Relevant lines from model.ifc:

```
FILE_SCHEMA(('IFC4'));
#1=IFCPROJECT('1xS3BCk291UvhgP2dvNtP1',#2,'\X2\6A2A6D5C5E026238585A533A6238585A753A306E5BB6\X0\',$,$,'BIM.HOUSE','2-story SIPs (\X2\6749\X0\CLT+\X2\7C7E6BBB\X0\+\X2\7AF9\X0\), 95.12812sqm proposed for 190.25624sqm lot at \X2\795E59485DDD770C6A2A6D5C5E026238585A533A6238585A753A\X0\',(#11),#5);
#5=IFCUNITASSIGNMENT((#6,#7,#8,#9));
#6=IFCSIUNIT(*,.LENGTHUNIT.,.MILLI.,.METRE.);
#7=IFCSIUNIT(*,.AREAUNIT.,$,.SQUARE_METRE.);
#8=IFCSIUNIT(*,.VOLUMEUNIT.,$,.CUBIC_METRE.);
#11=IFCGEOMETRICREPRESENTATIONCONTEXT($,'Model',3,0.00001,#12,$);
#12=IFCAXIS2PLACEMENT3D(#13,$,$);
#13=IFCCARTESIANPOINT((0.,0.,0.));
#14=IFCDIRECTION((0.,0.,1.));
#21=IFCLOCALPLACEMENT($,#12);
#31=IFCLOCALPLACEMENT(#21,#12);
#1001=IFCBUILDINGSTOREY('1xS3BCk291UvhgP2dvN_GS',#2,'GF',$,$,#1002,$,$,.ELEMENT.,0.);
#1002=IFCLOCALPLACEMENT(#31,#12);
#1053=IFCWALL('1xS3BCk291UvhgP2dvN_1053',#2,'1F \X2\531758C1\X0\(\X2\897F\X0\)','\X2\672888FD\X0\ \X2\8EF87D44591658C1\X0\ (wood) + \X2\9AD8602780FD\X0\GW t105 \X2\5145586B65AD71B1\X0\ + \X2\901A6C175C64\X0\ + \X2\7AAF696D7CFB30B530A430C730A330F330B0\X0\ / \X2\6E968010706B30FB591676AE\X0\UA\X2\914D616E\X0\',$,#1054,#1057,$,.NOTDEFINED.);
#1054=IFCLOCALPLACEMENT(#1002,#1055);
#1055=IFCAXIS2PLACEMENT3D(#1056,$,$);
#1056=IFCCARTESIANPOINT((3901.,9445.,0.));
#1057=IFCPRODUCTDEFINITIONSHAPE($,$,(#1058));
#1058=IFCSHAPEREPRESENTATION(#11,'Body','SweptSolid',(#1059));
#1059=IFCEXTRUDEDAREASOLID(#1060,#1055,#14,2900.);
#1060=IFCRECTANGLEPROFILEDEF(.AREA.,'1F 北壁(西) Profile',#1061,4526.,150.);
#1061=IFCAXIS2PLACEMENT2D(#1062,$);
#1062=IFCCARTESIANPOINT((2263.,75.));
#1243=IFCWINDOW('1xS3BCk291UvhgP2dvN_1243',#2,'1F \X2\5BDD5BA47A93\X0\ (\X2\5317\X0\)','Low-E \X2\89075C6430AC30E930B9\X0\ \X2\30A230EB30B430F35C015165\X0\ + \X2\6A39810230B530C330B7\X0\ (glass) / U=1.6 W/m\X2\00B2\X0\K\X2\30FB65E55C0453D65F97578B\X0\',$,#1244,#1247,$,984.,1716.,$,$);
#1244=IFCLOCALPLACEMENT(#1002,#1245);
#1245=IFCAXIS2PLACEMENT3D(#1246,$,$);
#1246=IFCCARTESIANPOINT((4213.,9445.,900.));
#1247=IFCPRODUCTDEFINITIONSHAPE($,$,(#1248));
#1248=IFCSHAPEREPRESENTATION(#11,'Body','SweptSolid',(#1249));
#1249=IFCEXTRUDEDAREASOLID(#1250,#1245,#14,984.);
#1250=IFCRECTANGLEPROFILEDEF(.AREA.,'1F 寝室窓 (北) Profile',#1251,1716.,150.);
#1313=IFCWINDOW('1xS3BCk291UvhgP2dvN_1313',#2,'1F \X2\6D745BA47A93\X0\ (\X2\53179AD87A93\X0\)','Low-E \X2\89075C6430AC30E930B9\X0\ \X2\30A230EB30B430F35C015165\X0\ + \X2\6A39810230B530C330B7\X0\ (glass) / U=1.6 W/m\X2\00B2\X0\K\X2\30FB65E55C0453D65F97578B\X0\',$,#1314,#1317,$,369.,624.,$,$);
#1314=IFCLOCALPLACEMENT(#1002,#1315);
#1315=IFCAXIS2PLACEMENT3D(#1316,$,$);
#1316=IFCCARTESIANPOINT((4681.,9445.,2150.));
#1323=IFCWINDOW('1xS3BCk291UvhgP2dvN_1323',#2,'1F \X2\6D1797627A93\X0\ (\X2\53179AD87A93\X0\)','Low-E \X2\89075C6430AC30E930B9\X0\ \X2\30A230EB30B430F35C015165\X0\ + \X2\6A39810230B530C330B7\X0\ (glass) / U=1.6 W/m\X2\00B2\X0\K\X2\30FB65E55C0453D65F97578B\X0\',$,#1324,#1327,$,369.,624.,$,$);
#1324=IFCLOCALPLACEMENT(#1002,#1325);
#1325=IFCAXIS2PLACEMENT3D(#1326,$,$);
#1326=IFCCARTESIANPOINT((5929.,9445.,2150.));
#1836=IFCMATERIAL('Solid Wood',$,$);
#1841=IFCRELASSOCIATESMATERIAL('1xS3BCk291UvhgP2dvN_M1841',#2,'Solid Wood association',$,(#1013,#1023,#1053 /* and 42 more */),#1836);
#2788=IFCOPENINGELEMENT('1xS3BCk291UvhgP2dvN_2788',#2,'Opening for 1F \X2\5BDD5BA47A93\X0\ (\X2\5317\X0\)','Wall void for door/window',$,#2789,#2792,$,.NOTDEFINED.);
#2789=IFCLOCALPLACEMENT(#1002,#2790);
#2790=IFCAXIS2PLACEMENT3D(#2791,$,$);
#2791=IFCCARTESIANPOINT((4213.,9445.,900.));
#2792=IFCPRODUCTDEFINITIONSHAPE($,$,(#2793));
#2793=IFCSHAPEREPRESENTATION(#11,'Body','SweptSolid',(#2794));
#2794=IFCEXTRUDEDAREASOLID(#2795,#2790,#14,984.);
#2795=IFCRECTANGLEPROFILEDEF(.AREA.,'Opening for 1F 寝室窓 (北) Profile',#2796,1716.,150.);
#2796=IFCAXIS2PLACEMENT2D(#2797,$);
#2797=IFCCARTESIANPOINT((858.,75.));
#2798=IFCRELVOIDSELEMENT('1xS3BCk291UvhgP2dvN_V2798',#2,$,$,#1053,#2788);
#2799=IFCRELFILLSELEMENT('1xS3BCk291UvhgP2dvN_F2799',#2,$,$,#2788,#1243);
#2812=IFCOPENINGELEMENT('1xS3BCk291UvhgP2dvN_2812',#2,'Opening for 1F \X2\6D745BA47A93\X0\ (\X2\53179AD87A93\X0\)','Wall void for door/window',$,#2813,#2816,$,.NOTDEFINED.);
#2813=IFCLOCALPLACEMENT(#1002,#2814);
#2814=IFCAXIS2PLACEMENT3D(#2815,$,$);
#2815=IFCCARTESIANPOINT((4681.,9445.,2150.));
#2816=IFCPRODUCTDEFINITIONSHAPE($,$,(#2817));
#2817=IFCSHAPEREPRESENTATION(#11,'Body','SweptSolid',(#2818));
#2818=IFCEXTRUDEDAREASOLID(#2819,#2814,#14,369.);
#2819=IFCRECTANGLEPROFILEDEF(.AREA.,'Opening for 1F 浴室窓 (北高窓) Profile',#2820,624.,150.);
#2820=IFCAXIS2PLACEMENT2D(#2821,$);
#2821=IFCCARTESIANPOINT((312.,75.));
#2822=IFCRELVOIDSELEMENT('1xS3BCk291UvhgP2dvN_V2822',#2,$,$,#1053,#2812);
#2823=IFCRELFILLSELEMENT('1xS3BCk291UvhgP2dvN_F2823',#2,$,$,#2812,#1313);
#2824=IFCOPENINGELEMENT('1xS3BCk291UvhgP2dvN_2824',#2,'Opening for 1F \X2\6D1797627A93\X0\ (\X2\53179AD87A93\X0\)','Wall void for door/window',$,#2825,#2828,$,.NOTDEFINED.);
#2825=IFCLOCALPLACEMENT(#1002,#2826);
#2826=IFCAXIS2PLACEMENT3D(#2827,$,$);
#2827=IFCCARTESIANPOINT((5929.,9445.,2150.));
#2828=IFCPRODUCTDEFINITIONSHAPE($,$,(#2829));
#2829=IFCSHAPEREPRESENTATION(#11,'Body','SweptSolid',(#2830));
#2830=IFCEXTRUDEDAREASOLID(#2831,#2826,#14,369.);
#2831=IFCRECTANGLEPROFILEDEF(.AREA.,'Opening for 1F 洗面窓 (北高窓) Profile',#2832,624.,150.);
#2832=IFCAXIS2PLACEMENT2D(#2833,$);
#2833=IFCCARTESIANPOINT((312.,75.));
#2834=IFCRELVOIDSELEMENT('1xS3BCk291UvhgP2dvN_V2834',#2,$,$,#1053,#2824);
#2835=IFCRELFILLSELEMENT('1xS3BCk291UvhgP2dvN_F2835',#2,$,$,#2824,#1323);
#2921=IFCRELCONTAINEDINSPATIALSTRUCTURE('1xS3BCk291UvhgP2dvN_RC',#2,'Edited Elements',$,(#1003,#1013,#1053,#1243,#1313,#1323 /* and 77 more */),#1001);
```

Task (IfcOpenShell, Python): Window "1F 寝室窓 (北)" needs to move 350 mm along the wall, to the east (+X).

```python
import ifcopenshell
import ifcopenshell.api.geometry
import ifcopenshell.util.placement
import ifcopenshell.util.unit

model = ifcopenshell.open("model.ifc")
unit_scale = ifcopenshell.util.unit.calculate_unit_scale(model)

window = model.by_guid("1xS3BCk291UvhgP2dvN_1243")
opening = window.FillsVoids[0].RelatingOpeningElement
wall = opening.VoidsElements[0].RelatingBuildingElement

wall_matrix = ifcopenshell.util.placement.get_local_placement(wall.ObjectPlacement)
shift = wall_matrix[:3, 0] * 0.35 / unit_scale
before = ifcopenshell.util.placement.get_local_placement(window.ObjectPlacement)[:3, 3].copy()

# The window is not placed relative to its opening, so move both.
for product in (opening, window):
    matrix = ifcopenshell.util.placement.get_local_placement(product.ObjectPlacement)
    matrix[:3, 3] += shift
    ifcopenshell.api.geometry.edit_object_placement(model, product=product, matrix=matrix, is_si=False)

after = ifcopenshell.util.placement.get_local_placement(window.ObjectPlacement)[:3, 3]
print("window moved by", (after - before).round(3) + 0.0)

model.write("model_v2.ifc")
```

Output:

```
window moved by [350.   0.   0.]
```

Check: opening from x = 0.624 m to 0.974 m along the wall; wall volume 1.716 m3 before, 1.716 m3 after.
